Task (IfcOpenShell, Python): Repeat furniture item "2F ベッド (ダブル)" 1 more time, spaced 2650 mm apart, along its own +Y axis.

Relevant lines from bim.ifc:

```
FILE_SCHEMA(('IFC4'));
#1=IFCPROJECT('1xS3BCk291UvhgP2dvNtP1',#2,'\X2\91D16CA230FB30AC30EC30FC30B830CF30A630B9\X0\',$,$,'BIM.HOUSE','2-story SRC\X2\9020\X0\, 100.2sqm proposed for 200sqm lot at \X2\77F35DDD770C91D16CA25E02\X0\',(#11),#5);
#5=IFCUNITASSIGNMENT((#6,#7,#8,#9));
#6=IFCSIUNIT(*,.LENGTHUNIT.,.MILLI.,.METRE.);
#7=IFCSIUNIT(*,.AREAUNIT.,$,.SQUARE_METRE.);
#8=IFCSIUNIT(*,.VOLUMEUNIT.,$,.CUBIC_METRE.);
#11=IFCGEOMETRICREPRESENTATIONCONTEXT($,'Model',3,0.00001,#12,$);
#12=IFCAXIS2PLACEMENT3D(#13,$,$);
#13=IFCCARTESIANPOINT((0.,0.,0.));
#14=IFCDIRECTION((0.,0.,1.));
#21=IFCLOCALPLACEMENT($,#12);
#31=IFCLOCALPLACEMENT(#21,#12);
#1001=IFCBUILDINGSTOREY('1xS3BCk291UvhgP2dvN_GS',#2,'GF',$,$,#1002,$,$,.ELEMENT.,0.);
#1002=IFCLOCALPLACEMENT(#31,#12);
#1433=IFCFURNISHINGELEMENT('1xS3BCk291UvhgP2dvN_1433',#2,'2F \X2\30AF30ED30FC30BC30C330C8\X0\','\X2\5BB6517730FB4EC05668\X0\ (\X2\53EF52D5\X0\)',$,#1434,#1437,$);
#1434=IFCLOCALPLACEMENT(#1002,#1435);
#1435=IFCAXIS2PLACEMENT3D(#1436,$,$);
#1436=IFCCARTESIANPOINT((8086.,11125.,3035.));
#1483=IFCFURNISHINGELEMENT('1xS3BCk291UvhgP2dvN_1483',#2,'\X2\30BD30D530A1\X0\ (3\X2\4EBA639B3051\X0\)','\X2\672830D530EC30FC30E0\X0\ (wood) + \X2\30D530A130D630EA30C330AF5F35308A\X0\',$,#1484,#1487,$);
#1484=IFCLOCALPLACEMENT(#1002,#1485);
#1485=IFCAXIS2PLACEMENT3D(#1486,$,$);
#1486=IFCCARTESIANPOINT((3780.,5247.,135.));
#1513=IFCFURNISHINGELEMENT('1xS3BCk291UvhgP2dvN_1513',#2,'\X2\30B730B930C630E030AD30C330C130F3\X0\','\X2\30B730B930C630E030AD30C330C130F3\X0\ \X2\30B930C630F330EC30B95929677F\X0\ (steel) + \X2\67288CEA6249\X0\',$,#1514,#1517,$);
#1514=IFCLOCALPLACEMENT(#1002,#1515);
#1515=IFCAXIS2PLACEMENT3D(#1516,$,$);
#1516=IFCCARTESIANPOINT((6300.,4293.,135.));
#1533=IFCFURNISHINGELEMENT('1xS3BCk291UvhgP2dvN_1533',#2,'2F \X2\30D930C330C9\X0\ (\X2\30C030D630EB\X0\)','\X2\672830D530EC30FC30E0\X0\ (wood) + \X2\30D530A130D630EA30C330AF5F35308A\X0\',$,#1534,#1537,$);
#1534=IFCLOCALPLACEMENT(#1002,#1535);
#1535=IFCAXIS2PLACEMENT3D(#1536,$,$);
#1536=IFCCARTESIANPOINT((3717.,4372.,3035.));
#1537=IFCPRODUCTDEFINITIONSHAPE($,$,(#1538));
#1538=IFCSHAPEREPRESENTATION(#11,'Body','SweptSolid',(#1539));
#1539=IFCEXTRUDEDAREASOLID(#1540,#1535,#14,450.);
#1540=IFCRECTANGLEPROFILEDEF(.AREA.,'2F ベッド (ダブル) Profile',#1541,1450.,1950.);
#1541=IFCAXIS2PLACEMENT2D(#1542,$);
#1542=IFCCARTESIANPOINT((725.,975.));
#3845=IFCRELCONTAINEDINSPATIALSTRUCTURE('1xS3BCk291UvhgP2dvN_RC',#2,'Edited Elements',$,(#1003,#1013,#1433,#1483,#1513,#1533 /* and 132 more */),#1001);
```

```python
import ifcopenshell
import ifcopenshell.api.geometry
import ifcopenshell.api.root
import ifcopenshell.util.element
import ifcopenshell.util.placement
import ifcopenshell.util.unit

model = ifcopenshell.open("bim.ifc")
unit_scale = ifcopenshell.util.unit.calculate_unit_scale(model)


def reuse_history(source, copy):
    """copy_class also copies each property set's owner history, people and application; keep the originals."""
    for rel in copy.IsDefinedBy:
        if rel.is_a("IfcRelDefinesByProperties") and (history := rel.RelatingPropertyDefinition.OwnerHistory):
            rel.RelatingPropertyDefinition.OwnerHistory = source.OwnerHistory
            ifcopenshell.util.element.remove_deep2(model, history)


source = model.by_id(1533)
base = ifcopenshell.util.placement.get_local_placement(source.ObjectPlacement)
step = base[:3, 1] * 2.65 / unit_scale

for i in range(1, 2):
    copy = ifcopenshell.api.root.copy_class(model, product=source)
    copy.Representation = ifcopenshell.util.element.copy_deep(
        model, source.Representation, exclude=["IfcGeometricRepresentationContext", "IfcRepresentationMap"]
    )
    reuse_history(source, copy)
    matrix = base.copy()
    matrix[:3, 3] += i * step
    print("added at", matrix[:3, 3].round(3) + 0.0)
    ifcopenshell.api.geometry.edit_object_placement(model, product=copy, matrix=matrix, is_si=False)

model.write("bim_updated.ifc")
```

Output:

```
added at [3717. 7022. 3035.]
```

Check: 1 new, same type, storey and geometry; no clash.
